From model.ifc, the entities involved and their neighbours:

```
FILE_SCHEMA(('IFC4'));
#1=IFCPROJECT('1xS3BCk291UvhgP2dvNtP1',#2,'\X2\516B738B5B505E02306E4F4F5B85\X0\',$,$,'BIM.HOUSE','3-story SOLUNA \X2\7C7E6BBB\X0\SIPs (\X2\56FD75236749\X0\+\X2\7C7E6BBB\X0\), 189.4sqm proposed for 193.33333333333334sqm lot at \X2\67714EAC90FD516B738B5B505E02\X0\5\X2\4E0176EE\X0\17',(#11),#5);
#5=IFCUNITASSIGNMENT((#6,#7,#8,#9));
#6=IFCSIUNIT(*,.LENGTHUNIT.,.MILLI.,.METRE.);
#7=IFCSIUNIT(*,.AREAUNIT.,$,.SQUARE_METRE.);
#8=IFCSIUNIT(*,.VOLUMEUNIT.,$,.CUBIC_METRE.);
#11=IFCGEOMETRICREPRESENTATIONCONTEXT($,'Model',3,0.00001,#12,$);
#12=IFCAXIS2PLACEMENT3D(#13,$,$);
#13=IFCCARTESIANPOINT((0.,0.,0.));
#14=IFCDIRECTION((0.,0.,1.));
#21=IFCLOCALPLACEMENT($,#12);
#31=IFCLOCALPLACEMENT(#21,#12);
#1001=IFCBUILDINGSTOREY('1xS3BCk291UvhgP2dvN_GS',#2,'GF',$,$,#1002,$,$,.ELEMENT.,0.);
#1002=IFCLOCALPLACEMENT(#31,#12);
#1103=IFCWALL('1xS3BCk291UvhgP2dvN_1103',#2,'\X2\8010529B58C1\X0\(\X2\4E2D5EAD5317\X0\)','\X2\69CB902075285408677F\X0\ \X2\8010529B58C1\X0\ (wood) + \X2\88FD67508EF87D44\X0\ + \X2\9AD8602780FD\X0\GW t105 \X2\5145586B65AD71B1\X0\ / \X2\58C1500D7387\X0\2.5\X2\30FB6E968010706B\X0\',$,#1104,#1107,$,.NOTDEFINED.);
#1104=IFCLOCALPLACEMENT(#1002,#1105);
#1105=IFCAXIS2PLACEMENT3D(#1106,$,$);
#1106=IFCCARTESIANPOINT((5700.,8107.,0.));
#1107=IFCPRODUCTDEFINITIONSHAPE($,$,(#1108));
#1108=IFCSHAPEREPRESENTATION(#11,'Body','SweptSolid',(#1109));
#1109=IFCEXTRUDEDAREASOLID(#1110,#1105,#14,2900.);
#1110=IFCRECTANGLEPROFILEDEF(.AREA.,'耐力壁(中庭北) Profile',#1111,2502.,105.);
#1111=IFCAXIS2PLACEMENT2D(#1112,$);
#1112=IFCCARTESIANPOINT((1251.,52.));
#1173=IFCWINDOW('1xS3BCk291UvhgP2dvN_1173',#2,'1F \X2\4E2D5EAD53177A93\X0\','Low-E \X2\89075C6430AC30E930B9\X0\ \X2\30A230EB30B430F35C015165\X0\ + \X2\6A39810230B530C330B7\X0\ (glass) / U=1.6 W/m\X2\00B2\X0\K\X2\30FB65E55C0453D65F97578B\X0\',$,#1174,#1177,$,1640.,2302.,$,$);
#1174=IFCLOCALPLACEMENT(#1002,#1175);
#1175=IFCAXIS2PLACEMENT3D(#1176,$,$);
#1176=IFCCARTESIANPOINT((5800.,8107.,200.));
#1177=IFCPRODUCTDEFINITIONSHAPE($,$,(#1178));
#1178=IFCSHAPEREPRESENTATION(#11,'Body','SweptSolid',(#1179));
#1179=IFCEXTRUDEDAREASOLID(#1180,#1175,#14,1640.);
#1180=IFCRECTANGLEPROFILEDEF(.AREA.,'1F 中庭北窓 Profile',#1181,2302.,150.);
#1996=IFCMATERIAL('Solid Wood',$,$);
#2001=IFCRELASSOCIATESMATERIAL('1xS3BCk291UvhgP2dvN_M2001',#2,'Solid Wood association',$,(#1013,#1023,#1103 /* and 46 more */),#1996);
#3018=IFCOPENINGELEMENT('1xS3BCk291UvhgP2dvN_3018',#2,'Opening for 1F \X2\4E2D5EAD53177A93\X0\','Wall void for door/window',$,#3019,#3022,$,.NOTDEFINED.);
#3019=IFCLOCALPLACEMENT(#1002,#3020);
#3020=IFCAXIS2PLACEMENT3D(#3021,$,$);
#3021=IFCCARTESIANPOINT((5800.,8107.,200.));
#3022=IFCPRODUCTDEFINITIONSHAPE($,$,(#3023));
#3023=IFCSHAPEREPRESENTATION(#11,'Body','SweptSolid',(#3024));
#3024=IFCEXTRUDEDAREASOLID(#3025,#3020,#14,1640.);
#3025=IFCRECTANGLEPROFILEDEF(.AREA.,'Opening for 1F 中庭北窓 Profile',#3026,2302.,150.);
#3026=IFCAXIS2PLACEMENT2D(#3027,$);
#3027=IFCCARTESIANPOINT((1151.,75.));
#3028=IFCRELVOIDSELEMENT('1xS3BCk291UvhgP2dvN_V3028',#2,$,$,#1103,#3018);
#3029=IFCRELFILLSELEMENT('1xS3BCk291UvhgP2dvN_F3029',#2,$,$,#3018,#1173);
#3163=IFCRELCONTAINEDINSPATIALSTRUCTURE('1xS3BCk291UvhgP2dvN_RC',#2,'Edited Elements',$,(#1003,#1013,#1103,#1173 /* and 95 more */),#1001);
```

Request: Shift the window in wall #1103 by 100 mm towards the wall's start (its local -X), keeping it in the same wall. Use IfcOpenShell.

```python
import ifcopenshell
import ifcopenshell.api.geometry
import ifcopenshell.util.placement
import ifcopenshell.util.unit

model = ifcopenshell.open("model.ifc")
unit_scale = ifcopenshell.util.unit.calculate_unit_scale(model)

window = model.by_id(1173)
opening = window.FillsVoids[0].RelatingOpeningElement
wall = opening.VoidsElements[0].RelatingBuildingElement

wall_matrix = ifcopenshell.util.placement.get_local_placement(wall.ObjectPlacement)
shift = wall_matrix[:3, 0] * -0.1 / unit_scale
before = ifcopenshell.util.placement.get_local_placement(window.ObjectPlacement)[:3, 3].copy()

# The window is not placed relative to its opening, so move both.
for product in (opening, window):
    matrix = ifcopenshell.util.placement.get_local_placement(product.ObjectPlacement)
    matrix[:3, 3] += shift
    ifcopenshell.api.geometry.edit_object_placement(model, product=product, matrix=matrix, is_si=False)

after = ifcopenshell.util.placement.get_local_placement(window.ObjectPlacement)[:3, 3]
print("window moved by", (after - before).round(3) + 0.0)

model.write("model_rev.ifc")
```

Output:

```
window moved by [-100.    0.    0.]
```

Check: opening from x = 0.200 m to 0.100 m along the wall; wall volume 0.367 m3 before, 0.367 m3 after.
